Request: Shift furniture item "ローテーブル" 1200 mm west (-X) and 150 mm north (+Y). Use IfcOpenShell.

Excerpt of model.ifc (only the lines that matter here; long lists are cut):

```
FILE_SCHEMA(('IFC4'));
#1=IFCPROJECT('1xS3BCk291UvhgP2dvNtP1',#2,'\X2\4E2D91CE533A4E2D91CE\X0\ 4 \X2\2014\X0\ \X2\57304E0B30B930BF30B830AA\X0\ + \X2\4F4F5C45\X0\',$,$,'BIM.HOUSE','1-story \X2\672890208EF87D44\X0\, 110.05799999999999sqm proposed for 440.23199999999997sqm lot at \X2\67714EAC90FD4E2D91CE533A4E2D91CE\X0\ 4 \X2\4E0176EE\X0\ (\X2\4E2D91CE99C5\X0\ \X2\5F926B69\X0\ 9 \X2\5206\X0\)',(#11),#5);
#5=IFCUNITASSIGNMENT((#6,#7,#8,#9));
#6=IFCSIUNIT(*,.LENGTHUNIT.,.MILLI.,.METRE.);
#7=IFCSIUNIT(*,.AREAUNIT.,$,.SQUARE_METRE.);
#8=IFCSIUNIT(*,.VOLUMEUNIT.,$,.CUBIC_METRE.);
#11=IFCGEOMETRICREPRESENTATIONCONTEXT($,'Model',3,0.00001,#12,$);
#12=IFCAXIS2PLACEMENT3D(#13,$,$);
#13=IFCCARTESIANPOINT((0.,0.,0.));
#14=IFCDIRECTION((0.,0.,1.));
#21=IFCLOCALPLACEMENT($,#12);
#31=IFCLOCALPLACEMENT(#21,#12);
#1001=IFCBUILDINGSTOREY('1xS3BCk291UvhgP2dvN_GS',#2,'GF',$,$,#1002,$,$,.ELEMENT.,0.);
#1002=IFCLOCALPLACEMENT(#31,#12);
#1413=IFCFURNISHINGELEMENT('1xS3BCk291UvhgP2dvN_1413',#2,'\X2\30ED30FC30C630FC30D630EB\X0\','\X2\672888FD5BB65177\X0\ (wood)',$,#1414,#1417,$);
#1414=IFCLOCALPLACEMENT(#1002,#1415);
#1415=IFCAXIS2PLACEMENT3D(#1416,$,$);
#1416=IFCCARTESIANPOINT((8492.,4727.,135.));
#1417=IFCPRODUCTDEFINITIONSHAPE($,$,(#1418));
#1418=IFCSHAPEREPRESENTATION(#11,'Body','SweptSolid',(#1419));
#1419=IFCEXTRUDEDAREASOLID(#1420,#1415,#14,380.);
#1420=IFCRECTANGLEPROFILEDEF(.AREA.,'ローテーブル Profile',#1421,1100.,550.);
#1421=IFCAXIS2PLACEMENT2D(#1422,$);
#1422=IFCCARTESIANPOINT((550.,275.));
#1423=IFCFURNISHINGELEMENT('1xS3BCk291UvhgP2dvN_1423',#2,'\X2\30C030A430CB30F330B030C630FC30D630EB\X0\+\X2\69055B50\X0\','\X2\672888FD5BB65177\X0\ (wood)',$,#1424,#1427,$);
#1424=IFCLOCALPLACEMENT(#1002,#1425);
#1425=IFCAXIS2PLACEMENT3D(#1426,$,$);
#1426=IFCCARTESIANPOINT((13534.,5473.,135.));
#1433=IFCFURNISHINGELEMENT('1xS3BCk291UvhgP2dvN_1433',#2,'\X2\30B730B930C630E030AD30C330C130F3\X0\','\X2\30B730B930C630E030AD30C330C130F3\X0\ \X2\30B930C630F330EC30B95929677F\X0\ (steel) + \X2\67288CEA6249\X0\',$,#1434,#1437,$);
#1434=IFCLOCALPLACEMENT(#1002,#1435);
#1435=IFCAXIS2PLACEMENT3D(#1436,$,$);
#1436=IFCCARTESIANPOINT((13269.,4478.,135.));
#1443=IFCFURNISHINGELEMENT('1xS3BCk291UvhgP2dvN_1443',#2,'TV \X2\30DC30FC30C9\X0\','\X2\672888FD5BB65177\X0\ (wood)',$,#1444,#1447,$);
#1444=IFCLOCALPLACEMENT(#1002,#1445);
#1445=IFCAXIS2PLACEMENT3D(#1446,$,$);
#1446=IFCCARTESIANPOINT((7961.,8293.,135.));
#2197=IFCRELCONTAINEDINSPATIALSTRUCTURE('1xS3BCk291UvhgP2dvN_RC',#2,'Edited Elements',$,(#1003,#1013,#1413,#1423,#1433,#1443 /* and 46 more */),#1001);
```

```python
import ifcopenshell
import ifcopenshell.api.geometry
import ifcopenshell.util.placement
import ifcopenshell.util.unit

model = ifcopenshell.open("model.ifc")
unit_scale = ifcopenshell.util.unit.calculate_unit_scale(model)

item = model.by_guid("1xS3BCk291UvhgP2dvN_1413")
matrix = ifcopenshell.util.placement.get_local_placement(item.ObjectPlacement)
matrix[0, 3] -= 1.2 / unit_scale
matrix[1, 3] += 0.15 / unit_scale
ifcopenshell.api.geometry.edit_object_placement(model, product=item, matrix=matrix, is_si=False)

print(ifcopenshell.util.placement.get_local_placement(item.ObjectPlacement).round(3) + 0.0)

model.write("model_edited.ifc")
```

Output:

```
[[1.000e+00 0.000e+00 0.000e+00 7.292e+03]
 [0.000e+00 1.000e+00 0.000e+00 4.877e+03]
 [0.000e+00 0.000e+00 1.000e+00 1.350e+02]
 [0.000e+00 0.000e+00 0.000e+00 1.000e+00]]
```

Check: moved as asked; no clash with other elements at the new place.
